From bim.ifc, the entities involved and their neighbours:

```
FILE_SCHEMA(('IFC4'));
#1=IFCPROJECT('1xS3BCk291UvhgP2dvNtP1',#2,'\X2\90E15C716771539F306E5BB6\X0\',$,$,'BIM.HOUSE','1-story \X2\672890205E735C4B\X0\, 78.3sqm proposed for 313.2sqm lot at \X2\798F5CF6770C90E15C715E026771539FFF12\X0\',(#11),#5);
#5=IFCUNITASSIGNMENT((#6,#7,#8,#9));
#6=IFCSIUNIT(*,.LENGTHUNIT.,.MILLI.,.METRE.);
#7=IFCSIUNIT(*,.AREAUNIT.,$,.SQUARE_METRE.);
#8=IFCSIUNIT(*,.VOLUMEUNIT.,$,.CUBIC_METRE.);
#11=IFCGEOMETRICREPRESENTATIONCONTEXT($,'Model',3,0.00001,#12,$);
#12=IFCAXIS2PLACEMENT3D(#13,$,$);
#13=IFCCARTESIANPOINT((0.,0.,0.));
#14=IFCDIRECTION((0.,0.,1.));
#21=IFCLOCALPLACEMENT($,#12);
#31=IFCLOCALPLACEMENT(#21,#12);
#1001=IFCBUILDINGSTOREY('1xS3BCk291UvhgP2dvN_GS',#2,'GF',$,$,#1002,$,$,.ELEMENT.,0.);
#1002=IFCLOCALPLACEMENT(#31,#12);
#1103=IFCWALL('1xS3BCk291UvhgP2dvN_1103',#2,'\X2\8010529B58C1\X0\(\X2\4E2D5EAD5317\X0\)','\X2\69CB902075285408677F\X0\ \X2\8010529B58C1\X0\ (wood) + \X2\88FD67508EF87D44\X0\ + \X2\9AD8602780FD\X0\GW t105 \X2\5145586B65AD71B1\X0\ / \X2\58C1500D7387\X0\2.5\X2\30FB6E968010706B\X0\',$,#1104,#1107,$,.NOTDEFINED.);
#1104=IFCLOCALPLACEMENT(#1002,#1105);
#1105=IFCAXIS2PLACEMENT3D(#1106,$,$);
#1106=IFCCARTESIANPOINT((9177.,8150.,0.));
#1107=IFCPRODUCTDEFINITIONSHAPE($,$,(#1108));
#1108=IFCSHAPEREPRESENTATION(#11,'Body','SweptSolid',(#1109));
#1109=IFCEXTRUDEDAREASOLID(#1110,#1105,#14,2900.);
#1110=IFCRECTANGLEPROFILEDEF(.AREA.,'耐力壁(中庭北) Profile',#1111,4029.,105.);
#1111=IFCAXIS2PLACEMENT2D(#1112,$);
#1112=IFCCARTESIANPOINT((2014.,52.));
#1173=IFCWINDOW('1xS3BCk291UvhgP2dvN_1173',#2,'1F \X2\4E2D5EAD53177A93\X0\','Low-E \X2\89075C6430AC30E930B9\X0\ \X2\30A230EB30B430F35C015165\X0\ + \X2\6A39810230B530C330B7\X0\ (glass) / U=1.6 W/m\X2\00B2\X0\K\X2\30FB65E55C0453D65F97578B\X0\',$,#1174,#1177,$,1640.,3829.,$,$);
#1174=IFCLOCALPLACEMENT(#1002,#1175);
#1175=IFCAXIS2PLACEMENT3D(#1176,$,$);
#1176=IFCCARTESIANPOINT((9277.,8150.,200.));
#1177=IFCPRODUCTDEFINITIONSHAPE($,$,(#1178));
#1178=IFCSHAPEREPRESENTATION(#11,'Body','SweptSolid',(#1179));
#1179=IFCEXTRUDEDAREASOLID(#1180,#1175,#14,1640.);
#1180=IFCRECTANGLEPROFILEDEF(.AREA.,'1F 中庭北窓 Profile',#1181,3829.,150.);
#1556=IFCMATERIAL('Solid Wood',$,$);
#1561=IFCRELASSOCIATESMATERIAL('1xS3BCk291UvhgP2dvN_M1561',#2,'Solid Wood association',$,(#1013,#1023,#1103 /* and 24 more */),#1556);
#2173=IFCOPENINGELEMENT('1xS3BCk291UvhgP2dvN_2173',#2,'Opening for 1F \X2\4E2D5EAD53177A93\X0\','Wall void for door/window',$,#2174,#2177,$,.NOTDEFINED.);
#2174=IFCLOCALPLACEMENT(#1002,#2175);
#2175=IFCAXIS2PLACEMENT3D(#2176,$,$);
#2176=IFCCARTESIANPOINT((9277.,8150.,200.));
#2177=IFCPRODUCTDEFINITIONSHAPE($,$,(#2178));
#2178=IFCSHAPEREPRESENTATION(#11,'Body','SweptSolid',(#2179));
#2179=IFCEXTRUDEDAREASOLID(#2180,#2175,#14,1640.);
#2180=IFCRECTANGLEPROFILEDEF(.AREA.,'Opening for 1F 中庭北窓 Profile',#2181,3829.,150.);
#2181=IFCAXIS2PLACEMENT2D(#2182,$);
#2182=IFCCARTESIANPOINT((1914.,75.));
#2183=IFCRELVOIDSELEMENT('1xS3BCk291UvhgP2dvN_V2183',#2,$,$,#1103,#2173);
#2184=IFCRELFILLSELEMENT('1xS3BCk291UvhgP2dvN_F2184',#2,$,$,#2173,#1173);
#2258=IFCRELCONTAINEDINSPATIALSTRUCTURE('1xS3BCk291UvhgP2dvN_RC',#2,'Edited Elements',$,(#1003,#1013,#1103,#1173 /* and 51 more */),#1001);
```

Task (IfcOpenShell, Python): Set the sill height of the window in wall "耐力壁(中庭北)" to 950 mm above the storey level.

```python
import numpy as np
import ifcopenshell
import ifcopenshell.api.geometry
import ifcopenshell.geom
import ifcopenshell.util.element
import ifcopenshell.util.placement
import ifcopenshell.util.shape
import ifcopenshell.util.unit

model = ifcopenshell.open("bim.ifc")
unit_scale = ifcopenshell.util.unit.calculate_unit_scale(model)

window = model.by_guid("1xS3BCk291UvhgP2dvN_1173")
opening = window.FillsVoids[0].RelatingOpeningElement
storey = ifcopenshell.util.element.get_container(window, ifc_class="IfcBuildingStorey")
level = ifcopenshell.util.placement.get_local_placement(storey.ObjectPlacement)[2, 3]

# The opening's origin need not be at the sill, so measure its lowest point.
shape = ifcopenshell.geom.create_shape(ifcopenshell.geom.settings(), opening)
bottom = ifcopenshell.util.shape.get_shape_bottom_elevation(shape, shape.geometry) / unit_scale
dz = level + 950.0 - bottom

shift = np.array([0.0, 0.0, dz])
# The window is not placed relative to its opening, so move both.
for product in (opening, window):
    matrix = ifcopenshell.util.placement.get_local_placement(product.ObjectPlacement)
    matrix[:3, 3] += shift
    ifcopenshell.api.geometry.edit_object_placement(model, product=product, matrix=matrix, is_si=False)

print(f"moved by {dz * unit_scale:+.3f} m")

model.write("bim_edited.ifc")
```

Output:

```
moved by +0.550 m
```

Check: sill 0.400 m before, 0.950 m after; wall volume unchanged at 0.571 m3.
